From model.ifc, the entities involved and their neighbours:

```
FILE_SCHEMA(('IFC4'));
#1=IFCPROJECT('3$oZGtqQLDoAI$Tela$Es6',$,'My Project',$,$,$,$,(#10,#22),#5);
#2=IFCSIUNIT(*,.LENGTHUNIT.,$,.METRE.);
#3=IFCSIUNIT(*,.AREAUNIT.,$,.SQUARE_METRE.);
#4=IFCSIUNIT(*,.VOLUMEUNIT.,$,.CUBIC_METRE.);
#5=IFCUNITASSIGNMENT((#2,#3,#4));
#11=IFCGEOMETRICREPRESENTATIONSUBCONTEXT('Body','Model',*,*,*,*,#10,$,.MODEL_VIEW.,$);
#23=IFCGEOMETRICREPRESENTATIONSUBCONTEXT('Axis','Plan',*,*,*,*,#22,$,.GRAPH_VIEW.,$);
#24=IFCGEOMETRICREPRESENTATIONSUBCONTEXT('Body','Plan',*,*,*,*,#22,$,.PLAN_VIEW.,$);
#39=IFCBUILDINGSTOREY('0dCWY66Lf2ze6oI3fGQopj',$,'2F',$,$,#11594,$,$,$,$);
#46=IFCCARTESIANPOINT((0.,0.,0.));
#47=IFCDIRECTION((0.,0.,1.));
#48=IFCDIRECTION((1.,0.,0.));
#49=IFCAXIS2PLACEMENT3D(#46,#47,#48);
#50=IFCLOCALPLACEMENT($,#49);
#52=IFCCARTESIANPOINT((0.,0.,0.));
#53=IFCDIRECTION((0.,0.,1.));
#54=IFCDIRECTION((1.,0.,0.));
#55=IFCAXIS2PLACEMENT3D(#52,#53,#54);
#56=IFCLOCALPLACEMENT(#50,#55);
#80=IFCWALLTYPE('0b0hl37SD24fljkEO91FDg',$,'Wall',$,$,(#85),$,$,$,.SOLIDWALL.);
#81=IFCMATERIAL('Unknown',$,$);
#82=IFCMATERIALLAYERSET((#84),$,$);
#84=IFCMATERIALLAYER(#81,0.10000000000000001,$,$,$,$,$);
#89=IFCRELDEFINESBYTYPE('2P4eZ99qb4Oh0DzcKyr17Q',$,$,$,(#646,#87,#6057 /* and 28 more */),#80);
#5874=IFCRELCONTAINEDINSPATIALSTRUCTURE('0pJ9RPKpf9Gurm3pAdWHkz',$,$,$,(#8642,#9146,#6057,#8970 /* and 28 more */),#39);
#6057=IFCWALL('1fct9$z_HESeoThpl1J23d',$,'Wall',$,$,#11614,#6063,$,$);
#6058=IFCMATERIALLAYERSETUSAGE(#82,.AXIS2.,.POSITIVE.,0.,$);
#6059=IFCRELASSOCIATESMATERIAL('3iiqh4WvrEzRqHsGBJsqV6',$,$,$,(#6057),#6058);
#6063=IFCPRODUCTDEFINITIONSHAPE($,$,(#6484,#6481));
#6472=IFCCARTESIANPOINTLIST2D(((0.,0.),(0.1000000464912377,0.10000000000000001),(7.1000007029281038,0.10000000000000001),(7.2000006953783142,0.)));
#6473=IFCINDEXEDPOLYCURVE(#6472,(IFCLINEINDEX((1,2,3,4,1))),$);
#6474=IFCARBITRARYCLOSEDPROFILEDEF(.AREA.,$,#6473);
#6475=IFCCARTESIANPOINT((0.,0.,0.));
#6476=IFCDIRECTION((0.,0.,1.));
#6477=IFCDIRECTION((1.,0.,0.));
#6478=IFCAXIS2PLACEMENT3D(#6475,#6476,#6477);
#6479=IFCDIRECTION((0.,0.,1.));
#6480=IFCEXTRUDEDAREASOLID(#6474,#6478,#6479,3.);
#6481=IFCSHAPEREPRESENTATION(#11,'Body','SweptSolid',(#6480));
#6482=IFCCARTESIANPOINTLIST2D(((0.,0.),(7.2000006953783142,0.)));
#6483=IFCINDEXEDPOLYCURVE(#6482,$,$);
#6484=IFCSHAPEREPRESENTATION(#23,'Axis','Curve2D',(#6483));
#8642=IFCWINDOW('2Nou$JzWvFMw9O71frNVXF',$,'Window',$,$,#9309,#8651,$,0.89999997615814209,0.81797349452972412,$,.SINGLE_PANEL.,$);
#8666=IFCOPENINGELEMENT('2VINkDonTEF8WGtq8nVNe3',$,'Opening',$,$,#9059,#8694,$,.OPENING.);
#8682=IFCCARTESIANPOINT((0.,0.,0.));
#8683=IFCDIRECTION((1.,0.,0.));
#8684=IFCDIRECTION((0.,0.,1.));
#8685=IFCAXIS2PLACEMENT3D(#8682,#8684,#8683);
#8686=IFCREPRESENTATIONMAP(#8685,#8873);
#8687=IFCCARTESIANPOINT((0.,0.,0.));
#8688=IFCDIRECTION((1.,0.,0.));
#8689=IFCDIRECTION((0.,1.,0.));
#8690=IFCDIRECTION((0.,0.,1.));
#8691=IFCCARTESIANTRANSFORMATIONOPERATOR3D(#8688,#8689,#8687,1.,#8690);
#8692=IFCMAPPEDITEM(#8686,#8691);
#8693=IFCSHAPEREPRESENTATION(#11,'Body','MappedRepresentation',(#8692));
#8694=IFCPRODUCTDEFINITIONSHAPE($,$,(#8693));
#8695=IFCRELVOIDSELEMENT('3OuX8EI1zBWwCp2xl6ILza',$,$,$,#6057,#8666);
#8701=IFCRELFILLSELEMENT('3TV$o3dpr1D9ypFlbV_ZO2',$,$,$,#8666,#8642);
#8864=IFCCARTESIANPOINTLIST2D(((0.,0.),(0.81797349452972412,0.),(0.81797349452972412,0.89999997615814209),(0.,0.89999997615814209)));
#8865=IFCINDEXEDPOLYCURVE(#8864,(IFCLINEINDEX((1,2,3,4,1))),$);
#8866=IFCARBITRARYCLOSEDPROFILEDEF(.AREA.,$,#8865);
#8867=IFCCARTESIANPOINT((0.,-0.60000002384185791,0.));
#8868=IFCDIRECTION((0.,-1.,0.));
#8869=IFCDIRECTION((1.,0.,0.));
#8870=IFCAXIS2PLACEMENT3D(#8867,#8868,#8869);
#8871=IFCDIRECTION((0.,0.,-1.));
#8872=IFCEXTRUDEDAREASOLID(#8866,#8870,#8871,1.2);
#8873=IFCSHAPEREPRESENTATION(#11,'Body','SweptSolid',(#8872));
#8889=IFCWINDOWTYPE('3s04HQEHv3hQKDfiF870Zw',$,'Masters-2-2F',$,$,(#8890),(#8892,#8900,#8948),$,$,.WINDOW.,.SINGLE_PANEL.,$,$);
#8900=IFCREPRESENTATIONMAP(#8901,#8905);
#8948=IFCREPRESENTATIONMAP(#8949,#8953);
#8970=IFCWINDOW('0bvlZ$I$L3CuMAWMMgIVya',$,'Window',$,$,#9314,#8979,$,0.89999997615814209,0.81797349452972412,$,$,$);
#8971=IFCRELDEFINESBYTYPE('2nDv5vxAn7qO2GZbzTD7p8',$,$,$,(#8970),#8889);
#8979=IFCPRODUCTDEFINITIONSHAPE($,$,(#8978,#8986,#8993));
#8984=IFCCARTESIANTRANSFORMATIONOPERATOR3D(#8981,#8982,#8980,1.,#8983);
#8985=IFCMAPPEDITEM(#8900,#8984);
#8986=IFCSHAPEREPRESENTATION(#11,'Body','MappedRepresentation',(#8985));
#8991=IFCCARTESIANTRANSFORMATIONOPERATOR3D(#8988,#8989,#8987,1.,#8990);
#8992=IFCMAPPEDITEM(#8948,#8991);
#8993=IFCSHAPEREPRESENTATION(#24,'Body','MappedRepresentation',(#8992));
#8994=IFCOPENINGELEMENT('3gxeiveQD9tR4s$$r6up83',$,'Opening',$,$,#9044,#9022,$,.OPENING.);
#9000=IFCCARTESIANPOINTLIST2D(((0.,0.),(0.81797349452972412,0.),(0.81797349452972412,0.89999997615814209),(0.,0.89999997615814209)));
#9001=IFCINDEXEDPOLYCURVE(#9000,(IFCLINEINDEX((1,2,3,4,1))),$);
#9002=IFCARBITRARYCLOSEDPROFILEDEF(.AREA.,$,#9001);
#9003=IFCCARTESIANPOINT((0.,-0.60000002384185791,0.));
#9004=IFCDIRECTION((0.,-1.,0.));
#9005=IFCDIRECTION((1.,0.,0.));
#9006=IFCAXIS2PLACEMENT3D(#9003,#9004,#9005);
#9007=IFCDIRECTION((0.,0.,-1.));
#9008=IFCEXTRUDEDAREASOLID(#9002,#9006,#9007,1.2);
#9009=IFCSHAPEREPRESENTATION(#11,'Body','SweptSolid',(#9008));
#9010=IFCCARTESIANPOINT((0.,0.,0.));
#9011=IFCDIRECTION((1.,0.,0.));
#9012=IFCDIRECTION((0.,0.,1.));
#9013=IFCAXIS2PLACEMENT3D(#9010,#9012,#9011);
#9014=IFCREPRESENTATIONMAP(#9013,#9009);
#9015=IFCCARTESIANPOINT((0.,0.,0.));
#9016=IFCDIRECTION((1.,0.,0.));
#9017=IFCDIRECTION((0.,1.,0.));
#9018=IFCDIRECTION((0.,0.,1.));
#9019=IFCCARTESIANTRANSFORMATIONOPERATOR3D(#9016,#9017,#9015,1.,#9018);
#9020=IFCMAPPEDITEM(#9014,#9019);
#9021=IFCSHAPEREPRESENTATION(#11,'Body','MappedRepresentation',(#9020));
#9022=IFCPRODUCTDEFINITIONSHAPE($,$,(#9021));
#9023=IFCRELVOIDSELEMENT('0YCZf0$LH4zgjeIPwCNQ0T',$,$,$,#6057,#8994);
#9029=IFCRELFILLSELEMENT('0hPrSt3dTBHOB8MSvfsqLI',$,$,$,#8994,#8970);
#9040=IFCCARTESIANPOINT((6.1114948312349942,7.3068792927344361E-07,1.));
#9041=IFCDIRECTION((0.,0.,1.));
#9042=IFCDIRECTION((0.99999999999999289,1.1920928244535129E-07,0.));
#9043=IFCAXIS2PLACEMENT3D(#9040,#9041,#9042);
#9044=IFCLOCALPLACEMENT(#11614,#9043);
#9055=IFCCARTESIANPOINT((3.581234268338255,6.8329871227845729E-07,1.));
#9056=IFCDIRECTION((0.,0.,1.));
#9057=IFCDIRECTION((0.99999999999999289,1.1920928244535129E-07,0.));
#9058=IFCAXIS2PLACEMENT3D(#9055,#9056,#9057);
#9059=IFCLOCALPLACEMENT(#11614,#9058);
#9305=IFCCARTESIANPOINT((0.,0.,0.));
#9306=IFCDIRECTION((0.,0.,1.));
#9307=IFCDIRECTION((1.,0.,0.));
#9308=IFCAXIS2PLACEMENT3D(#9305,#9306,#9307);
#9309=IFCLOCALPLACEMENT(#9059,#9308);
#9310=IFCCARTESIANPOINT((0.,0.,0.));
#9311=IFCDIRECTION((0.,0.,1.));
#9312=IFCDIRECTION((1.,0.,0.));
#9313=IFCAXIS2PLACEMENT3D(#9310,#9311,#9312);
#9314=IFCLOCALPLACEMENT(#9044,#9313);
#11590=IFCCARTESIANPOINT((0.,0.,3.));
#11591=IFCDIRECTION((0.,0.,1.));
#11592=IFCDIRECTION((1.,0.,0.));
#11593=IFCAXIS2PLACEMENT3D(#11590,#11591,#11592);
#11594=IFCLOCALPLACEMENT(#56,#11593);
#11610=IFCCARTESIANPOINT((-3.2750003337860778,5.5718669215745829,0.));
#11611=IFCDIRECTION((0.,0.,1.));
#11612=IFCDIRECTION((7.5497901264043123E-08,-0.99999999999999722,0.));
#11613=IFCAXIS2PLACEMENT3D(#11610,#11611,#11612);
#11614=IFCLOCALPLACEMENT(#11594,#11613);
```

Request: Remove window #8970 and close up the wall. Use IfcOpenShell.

```python
import ifcopenshell
import ifcopenshell.api.feature
import ifcopenshell.api.root
import ifcopenshell.geom
import ifcopenshell.util.shape

model = ifcopenshell.open("model.ifc")
settings = ifcopenshell.geom.settings()


def volume(element):
    """Net volume in cubic metres, openings subtracted."""
    shape = ifcopenshell.geom.create_shape(settings, element)
    return ifcopenshell.util.shape.get_volume(shape.geometry)


window = model.by_guid("0bvlZ$I$L3CuMAWMMgIVya")
opening = window.FillsVoids[0].RelatingOpeningElement
wall = opening.VoidsElements[0].RelatingBuildingElement
before = volume(wall)

ifcopenshell.api.root.remove_product(model, product=window)
ifcopenshell.api.feature.remove_feature(model, feature=opening)

after = volume(wall)

print(f"wall volume {before:.3f} -> {after:.3f} m3")

model.write("model_rev.ifc")
```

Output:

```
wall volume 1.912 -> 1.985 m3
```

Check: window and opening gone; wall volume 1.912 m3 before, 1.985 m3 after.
